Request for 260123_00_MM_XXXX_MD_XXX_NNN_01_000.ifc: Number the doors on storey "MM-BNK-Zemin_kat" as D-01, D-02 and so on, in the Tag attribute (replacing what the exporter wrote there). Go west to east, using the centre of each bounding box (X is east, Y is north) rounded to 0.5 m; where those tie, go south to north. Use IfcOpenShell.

First a look at what the model holds.

```python
import ifcopenshell
import ifcopenshell.util.element
import ifcopenshell.util.placement

model = ifcopenshell.open("260123_00_MM_XXXX_MD_XXX_NNN_01_000.ifc")
print(model.schema)
storey = next(s for s in model.by_type("IfcBuildingStorey") if s.Name == "MM-BNK-Zemin_kat")
doors = [e for e in ifcopenshell.util.element.get_decomposition(storey) if e.is_a("IfcDoor")]
for e in sorted(doors, key=lambda e: e.id()):
    origin = ifcopenshell.util.placement.get_local_placement(e.ObjectPlacement)[:3, 3]
    print(e.id(), e.Tag, e.Name, origin.round(2) + 0.0, sep=" | ")
```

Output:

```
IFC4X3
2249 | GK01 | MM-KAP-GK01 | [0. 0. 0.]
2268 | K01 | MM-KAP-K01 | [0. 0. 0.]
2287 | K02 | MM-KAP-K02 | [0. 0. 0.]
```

```python
import ifcopenshell
import ifcopenshell.geom
import ifcopenshell.util.element
import ifcopenshell.util.shape

model = ifcopenshell.open("260123_00_MM_XXXX_MD_XXX_NNN_01_000.ifc")
settings = ifcopenshell.geom.settings()
settings.set("use-world-coords", True)


def centre(element):
    shape = ifcopenshell.geom.create_shape(settings, element)
    return ifcopenshell.util.shape.get_bbox_centroid(shape.geometry)


storey = next(s for s in model.by_type("IfcBuildingStorey") if s.Name == "MM-BNK-Zemin_kat")
doors = [e for e in ifcopenshell.util.element.get_decomposition(storey) if e.is_a("IfcDoor")]

# Insertion points can sit at a corner or the storey origin, so sort by the geometry (in metres).
centres = {e: centre(e) for e in doors}
doors.sort(key=lambda e: (round(centres[e][0] / 0.5), centres[e][1]))

for i, e in enumerate(doors, start=1):
    number = f"D-{i:02d}"
    e.Tag = number
    print(e.id(), number)

model.write("260123_00_MM_XXXX_MD_XXX_NNN_01_000_edited.ifc")
```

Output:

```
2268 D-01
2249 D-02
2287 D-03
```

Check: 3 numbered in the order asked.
